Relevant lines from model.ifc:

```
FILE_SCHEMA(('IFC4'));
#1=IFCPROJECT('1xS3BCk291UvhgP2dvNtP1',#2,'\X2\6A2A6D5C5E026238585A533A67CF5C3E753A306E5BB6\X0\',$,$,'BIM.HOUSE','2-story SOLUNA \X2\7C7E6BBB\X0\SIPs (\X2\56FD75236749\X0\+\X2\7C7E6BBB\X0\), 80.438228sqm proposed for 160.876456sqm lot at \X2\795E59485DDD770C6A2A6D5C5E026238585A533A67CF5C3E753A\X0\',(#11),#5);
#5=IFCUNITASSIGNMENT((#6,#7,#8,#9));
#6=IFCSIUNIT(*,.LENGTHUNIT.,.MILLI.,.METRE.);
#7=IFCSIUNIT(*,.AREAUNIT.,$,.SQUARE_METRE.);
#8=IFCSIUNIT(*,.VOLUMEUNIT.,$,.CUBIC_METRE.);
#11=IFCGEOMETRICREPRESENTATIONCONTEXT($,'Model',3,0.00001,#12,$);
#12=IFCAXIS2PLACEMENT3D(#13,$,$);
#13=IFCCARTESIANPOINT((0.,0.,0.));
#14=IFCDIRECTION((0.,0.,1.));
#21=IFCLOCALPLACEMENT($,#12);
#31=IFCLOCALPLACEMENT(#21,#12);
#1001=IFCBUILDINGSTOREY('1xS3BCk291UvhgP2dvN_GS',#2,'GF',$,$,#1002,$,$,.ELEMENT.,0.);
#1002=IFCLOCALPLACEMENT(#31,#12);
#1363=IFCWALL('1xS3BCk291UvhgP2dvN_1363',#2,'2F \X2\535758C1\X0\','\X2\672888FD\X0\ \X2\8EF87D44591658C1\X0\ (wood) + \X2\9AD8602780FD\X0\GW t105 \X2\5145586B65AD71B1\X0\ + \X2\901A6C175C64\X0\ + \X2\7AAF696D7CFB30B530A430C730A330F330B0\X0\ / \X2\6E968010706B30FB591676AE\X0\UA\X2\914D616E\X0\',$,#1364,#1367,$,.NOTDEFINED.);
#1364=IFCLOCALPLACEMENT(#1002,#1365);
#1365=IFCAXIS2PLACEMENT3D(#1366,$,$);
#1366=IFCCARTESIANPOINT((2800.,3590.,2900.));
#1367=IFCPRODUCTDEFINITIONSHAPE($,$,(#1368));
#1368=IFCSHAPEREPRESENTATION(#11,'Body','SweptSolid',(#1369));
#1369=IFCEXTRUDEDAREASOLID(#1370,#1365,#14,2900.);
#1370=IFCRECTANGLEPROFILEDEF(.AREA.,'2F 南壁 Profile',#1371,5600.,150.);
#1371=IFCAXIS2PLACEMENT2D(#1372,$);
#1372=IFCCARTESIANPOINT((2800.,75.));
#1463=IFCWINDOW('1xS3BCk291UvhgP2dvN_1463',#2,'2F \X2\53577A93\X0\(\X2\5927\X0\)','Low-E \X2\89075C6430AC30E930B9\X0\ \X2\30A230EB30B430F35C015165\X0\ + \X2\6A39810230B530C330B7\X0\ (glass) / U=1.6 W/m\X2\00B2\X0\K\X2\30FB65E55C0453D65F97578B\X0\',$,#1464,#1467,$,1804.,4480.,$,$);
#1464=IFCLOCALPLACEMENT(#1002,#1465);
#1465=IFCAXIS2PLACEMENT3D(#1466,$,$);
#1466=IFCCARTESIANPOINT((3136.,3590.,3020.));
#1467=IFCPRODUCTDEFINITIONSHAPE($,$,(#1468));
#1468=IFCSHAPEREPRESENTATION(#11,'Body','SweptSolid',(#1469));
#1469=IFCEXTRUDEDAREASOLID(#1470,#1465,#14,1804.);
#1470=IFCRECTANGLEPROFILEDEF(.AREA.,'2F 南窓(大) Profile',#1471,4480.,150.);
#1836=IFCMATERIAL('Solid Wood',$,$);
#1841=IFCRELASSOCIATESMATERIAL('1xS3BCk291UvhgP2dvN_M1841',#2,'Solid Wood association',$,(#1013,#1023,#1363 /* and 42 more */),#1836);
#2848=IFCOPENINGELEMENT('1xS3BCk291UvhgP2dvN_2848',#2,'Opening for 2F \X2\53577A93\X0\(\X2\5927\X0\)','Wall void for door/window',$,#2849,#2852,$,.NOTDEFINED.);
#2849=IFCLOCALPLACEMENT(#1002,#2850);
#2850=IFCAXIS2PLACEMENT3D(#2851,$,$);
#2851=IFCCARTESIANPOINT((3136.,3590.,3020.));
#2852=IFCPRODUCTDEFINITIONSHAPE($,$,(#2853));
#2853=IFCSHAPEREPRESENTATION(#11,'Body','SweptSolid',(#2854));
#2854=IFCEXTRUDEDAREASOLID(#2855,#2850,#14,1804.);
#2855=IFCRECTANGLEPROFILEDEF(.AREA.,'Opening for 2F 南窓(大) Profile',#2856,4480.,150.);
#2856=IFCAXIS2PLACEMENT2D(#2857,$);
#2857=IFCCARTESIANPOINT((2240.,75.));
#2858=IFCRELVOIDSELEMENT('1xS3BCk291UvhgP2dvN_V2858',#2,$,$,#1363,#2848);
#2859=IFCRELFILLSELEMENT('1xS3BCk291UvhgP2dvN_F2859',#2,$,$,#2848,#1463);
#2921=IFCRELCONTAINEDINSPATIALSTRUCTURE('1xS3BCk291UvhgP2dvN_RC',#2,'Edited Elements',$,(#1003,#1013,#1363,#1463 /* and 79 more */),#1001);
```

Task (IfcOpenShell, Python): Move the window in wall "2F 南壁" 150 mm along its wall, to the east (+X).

```python
import ifcopenshell
import ifcopenshell.api.geometry
import ifcopenshell.util.placement
import ifcopenshell.util.unit

model = ifcopenshell.open("model.ifc")
unit_scale = ifcopenshell.util.unit.calculate_unit_scale(model)

window = model.by_guid("1xS3BCk291UvhgP2dvN_1463")
opening = window.FillsVoids[0].RelatingOpeningElement
wall = opening.VoidsElements[0].RelatingBuildingElement

wall_matrix = ifcopenshell.util.placement.get_local_placement(wall.ObjectPlacement)
shift = wall_matrix[:3, 0] * 0.15 / unit_scale
before = ifcopenshell.util.placement.get_local_placement(window.ObjectPlacement)[:3, 3].copy()

# The window is not placed relative to its opening, so move both.
for product in (opening, window):
    matrix = ifcopenshell.util.placement.get_local_placement(product.ObjectPlacement)
    matrix[:3, 3] += shift
    ifcopenshell.api.geometry.edit_object_placement(model, product=product, matrix=matrix, is_si=False)

after = ifcopenshell.util.placement.get_local_placement(window.ObjectPlacement)[:3, 3]
print("window moved by", (after - before).round(3) + 0.0)

model.write("model-out.ifc")
```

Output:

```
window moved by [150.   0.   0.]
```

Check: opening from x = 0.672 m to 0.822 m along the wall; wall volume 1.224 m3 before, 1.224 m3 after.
